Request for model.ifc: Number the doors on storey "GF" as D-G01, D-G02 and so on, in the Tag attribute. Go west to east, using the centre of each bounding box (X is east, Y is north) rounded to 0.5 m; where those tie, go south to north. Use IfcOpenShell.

First a look at what the model holds.

```python
import ifcopenshell
import ifcopenshell.util.element
import ifcopenshell.util.placement

model = ifcopenshell.open("model.ifc")
print(model.schema)
storey = next(s for s in model.by_type("IfcBuildingStorey") if s.Name == "GF")
doors = [e for e in ifcopenshell.util.element.get_decomposition(storey) if e.is_a("IfcDoor")]
for e in sorted(doors, key=lambda e: e.id()):
    origin = ifcopenshell.util.placement.get_local_placement(e.ObjectPlacement)[:3, 3]
    print(e.id(), e.Tag, e.Name, origin.round(2) + 0.0, sep=" | ")
```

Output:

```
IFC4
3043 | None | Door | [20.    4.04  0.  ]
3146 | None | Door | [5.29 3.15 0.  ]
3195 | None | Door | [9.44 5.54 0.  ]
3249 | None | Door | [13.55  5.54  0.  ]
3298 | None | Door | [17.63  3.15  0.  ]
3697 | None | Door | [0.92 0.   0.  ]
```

```python
import ifcopenshell
import ifcopenshell.geom
import ifcopenshell.util.element
import ifcopenshell.util.shape

model = ifcopenshell.open("model.ifc")
settings = ifcopenshell.geom.settings()
settings.set("use-world-coords", True)


def centre(element):
    shape = ifcopenshell.geom.create_shape(settings, element)
    return ifcopenshell.util.shape.get_bbox_centroid(shape.geometry)


storey = next(s for s in model.by_type("IfcBuildingStorey") if s.Name == "GF")
doors = [e for e in ifcopenshell.util.element.get_decomposition(storey) if e.is_a("IfcDoor")]

# Insertion points can sit at a corner or the storey origin, so sort by the geometry (in metres).
centres = {e: centre(e) for e in doors}
doors.sort(key=lambda e: (round(centres[e][0] / 0.5), centres[e][1]))

for i, e in enumerate(doors, start=1):
    number = f"D-G{i:02d}"
    e.Tag = number
    print(e.id(), number)

model.write("model_updated.ifc")
```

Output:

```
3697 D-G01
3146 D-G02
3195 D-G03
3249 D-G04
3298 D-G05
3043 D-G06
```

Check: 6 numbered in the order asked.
